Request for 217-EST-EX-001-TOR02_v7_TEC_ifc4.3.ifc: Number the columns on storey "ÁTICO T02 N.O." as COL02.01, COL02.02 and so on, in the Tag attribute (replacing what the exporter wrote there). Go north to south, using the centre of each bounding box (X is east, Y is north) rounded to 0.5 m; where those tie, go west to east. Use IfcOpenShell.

First a look at what the model holds.

```python
import ifcopenshell
import ifcopenshell.util.element
import ifcopenshell.util.placement

model = ifcopenshell.open("217-EST-EX-001-TOR02_v7_TEC_ifc4.3.ifc")
print(model.schema)
storey = next(s for s in model.by_type("IfcBuildingStorey") if s.Name == "ÁTICO T02 N.O.")
columns = [e for e in ifcopenshell.util.element.get_decomposition(storey) if e.is_a("IfcColumn")]
for e in sorted(columns, key=lambda e: e.id()):
    origin = ifcopenshell.util.placement.get_local_placement(e.ObjectPlacement)[:3, 3]
    print(e.id(), e.Tag, e.Name, origin.round(2) + 0.0, sep=" | ")
```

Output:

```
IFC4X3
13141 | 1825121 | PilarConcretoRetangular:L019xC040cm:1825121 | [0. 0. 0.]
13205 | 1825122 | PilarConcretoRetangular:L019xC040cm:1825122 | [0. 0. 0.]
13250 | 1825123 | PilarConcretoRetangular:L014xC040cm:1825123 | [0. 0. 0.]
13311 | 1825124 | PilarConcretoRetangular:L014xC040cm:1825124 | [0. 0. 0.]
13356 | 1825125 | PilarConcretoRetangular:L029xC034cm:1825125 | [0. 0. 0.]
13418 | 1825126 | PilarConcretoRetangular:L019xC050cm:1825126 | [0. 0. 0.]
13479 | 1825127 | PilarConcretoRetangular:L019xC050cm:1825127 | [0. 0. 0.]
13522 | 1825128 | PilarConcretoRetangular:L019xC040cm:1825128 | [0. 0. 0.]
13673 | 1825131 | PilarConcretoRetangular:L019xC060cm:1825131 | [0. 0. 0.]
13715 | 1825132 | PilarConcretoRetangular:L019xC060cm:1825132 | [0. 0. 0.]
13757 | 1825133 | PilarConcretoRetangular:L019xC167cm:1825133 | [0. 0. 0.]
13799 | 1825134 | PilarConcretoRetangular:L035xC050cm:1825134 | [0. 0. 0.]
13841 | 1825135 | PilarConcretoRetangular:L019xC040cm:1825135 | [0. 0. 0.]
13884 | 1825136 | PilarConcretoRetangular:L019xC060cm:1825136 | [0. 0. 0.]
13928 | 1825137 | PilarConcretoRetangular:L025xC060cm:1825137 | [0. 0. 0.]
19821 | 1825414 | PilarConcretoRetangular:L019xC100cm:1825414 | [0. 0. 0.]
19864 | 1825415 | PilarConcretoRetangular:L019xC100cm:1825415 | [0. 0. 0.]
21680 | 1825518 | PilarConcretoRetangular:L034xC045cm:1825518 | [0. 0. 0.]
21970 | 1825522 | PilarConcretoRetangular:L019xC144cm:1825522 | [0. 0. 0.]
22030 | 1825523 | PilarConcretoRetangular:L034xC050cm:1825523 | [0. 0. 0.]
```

```python
import ifcopenshell
import ifcopenshell.geom
import ifcopenshell.util.element
import ifcopenshell.util.shape

model = ifcopenshell.open("217-EST-EX-001-TOR02_v7_TEC_ifc4.3.ifc")
settings = ifcopenshell.geom.settings()
settings.set("use-world-coords", True)


def centre(element):
    shape = ifcopenshell.geom.create_shape(settings, element)
    return ifcopenshell.util.shape.get_bbox_centroid(shape.geometry)


storey = next(s for s in model.by_type("IfcBuildingStorey") if s.Name == "ÁTICO T02 N.O.")
columns = [e for e in ifcopenshell.util.element.get_decomposition(storey) if e.is_a("IfcColumn")]

# Insertion points can sit at a corner or the storey origin, so sort by the geometry (in metres).
centres = {e: centre(e) for e in columns}
columns.sort(key=lambda e: (-round(centres[e][1] / 0.5), centres[e][0]))

for i, e in enumerate(columns, start=1):
    number = f"COL02.{i:02d}"
    e.Tag = number
    print(e.id(), number)

model.write("217-EST-EX-001-TOR02_v7_TEC_ifc4.3_edited.ifc")
```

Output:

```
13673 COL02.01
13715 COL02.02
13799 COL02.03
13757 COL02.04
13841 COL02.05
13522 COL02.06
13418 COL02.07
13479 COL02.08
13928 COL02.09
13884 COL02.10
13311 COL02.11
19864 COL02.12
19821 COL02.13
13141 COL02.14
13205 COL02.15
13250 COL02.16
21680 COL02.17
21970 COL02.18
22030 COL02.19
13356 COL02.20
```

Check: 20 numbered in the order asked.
